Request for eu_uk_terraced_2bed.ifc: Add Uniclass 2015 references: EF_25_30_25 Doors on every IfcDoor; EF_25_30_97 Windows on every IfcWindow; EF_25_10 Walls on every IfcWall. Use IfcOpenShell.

First a look at what the model holds.

```python
import ifcopenshell

model = ifcopenshell.open("eu_uk_terraced_2bed.ifc")
print(model.schema)
print("classifications:", [c.Name for c in model.by_type("IfcClassification")])
for ifc_class in ("IfcDoor", "IfcRoof", "IfcStair", "IfcWall", "IfcWindow"):
    print(ifc_class, len(model.by_type(ifc_class)))
```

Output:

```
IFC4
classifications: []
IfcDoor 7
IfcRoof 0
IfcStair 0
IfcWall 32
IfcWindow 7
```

```python
import ifcopenshell
import ifcopenshell.api.classification

model = ifcopenshell.open("eu_uk_terraced_2bed.ifc")

system = ifcopenshell.api.classification.add_classification(model, classification="Uniclass 2015")

codes = {
    "IfcDoor": ("EF_25_30_25", "Doors"),
    "IfcWindow": ("EF_25_30_97", "Windows"),
    "IfcWall": ("EF_25_10", "Walls"),
}
for ifc_class, (code, name) in codes.items():
    products = model.by_type(ifc_class)
    ifcopenshell.api.classification.add_reference(
        model, products=products, classification=system, identification=code, name=name
    )
    print(code, len(products))

model.write("eu_uk_terraced_2bed_edited.ifc")
```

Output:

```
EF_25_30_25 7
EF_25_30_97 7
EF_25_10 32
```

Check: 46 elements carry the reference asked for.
